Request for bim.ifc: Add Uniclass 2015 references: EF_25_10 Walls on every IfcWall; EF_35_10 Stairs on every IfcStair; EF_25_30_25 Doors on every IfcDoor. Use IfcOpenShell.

First a look at what the model holds.

```python
import ifcopenshell

model = ifcopenshell.open("bim.ifc")
print(model.schema)
print("classifications:", [c.Name for c in model.by_type("IfcClassification")])
for ifc_class in ("IfcDoor", "IfcRoof", "IfcStair", "IfcWall", "IfcWindow"):
    print(ifc_class, len(model.by_type(ifc_class)))
```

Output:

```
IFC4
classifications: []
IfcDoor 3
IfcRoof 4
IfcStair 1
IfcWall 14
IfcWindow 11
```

```python
import ifcopenshell
import ifcopenshell.api.classification

model = ifcopenshell.open("bim.ifc")

system = ifcopenshell.api.classification.add_classification(model, classification="Uniclass 2015")

codes = {
    "IfcWall": ("EF_25_10", "Walls"),
    "IfcStair": ("EF_35_10", "Stairs"),
    "IfcDoor": ("EF_25_30_25", "Doors"),
}
for ifc_class, (code, name) in codes.items():
    products = model.by_type(ifc_class)
    ifcopenshell.api.classification.add_reference(
        model, products=products, classification=system, identification=code, name=name
    )
    print(code, len(products))

model.write("bim_updated.ifc")
```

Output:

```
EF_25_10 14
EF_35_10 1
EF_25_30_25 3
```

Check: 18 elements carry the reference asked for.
